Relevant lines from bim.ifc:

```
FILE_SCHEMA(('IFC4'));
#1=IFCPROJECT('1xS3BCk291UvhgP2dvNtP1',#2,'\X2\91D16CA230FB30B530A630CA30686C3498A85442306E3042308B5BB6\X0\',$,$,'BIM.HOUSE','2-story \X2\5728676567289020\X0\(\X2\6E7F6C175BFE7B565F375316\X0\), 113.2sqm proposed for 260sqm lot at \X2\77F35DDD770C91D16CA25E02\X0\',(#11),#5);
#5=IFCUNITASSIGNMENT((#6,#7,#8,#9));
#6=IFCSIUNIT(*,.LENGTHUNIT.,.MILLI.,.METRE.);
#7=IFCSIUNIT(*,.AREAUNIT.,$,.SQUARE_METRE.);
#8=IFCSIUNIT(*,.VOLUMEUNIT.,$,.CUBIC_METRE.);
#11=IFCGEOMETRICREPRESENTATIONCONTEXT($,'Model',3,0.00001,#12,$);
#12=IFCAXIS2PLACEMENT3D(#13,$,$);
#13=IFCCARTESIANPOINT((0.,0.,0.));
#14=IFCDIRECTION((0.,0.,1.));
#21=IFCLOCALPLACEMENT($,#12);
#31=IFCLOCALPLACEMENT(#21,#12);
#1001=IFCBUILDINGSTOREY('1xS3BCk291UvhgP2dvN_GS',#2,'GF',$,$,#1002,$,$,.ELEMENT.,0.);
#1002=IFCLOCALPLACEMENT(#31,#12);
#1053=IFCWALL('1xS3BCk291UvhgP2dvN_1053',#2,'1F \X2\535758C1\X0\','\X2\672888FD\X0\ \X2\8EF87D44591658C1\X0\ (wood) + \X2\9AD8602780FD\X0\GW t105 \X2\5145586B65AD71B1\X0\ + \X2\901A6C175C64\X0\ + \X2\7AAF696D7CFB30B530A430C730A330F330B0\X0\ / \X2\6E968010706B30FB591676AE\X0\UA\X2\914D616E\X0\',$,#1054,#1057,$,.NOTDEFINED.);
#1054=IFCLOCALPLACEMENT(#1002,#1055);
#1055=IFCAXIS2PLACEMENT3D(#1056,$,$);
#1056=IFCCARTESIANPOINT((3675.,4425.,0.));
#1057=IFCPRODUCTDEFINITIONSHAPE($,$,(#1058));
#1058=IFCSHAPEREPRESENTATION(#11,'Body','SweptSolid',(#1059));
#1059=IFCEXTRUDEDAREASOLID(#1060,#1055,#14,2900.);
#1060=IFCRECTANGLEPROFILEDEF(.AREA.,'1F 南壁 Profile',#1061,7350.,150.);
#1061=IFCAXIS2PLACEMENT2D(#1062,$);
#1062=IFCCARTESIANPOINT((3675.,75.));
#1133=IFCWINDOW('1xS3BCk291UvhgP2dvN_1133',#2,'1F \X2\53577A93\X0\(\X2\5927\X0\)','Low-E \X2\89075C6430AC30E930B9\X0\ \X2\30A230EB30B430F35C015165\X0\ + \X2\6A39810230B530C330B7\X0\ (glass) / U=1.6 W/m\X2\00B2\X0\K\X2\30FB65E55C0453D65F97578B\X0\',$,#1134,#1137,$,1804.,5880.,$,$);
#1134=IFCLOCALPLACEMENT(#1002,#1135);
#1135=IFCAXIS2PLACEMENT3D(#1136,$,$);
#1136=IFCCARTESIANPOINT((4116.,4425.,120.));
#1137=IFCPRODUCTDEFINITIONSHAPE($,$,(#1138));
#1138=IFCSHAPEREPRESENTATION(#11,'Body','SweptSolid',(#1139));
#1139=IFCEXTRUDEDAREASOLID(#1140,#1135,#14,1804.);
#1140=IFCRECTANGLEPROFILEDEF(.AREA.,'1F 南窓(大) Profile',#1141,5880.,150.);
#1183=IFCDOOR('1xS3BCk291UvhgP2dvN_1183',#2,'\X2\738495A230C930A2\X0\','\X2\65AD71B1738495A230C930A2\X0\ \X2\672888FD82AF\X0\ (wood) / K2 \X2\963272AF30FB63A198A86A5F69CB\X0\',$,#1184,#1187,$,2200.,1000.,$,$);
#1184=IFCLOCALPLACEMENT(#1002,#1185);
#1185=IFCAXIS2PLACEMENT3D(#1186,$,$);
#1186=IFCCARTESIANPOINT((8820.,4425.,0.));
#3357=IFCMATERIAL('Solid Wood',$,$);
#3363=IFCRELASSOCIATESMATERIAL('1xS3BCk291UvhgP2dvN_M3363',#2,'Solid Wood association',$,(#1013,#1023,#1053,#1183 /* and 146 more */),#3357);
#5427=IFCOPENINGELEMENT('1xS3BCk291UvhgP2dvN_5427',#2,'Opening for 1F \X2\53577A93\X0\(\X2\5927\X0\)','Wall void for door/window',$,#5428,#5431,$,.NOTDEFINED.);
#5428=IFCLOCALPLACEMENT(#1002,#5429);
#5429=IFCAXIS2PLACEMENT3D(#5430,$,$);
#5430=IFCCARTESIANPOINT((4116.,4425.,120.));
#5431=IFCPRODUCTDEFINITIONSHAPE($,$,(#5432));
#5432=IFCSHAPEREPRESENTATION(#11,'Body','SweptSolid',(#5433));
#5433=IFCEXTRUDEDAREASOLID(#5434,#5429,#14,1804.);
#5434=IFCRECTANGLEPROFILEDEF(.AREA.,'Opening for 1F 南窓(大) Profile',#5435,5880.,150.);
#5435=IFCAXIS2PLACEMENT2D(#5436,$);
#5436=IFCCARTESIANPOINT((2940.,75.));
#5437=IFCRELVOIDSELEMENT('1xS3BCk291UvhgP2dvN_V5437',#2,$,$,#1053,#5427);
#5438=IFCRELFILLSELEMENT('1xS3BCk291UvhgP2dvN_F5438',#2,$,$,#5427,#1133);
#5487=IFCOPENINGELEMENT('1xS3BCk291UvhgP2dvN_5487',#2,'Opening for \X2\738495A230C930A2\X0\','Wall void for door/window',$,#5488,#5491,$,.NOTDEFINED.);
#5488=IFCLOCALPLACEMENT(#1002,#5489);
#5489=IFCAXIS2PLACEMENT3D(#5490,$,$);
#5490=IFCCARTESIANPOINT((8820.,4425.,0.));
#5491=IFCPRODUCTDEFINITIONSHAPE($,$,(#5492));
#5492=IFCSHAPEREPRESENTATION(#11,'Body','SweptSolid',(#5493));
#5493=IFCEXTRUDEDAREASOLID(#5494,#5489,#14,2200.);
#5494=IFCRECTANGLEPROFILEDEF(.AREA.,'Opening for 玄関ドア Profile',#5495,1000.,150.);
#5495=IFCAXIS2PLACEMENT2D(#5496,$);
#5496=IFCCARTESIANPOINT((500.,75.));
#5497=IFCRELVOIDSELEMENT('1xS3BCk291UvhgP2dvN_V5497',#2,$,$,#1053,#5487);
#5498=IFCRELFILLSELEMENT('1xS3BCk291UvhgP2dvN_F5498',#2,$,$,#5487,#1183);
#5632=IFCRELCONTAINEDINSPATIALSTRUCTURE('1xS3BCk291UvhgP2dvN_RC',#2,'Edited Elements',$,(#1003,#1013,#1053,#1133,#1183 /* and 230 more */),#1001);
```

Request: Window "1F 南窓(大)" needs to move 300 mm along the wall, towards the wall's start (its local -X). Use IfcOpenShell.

```python
import ifcopenshell
import ifcopenshell.api.geometry
import ifcopenshell.util.placement
import ifcopenshell.util.unit

model = ifcopenshell.open("bim.ifc")
unit_scale = ifcopenshell.util.unit.calculate_unit_scale(model)

window = model.by_guid("1xS3BCk291UvhgP2dvN_1133")
opening = window.FillsVoids[0].RelatingOpeningElement
wall = opening.VoidsElements[0].RelatingBuildingElement

wall_matrix = ifcopenshell.util.placement.get_local_placement(wall.ObjectPlacement)
shift = wall_matrix[:3, 0] * -0.3 / unit_scale
before = ifcopenshell.util.placement.get_local_placement(window.ObjectPlacement)[:3, 3].copy()

# The window is not placed relative to its opening, so move both.
for product in (opening, window):
    matrix = ifcopenshell.util.placement.get_local_placement(product.ObjectPlacement)
    matrix[:3, 3] += shift
    ifcopenshell.api.geometry.edit_object_placement(model, product=product, matrix=matrix, is_si=False)

after = ifcopenshell.util.placement.get_local_placement(window.ObjectPlacement)[:3, 3]
print("window moved by", (after - before).round(3) + 0.0)

model.write("bim_v2.ifc")
```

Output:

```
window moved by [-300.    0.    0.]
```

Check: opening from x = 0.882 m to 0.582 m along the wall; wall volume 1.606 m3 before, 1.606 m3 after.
